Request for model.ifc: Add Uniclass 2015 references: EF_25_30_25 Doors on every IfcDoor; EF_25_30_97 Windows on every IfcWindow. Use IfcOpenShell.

First a look at what the model holds.

```python
import ifcopenshell

model = ifcopenshell.open("model.ifc")
print(model.schema)
print("classifications:", [c.Name for c in model.by_type("IfcClassification")])
for ifc_class in ("IfcDoor", "IfcRoof", "IfcStair", "IfcWall", "IfcWindow"):
    print(ifc_class, len(model.by_type(ifc_class)))
```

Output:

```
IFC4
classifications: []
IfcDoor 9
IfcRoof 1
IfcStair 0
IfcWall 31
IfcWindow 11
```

```python
import ifcopenshell
import ifcopenshell.api.classification

model = ifcopenshell.open("model.ifc")

system = ifcopenshell.api.classification.add_classification(model, classification="Uniclass 2015")

codes = {
    "IfcDoor": ("EF_25_30_25", "Doors"),
    "IfcWindow": ("EF_25_30_97", "Windows"),
}
for ifc_class, (code, name) in codes.items():
    products = model.by_type(ifc_class)
    ifcopenshell.api.classification.add_reference(
        model, products=products, classification=system, identification=code, name=name
    )
    print(code, len(products))

model.write("model_v2.ifc")
```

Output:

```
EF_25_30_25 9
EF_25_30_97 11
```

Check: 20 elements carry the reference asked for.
